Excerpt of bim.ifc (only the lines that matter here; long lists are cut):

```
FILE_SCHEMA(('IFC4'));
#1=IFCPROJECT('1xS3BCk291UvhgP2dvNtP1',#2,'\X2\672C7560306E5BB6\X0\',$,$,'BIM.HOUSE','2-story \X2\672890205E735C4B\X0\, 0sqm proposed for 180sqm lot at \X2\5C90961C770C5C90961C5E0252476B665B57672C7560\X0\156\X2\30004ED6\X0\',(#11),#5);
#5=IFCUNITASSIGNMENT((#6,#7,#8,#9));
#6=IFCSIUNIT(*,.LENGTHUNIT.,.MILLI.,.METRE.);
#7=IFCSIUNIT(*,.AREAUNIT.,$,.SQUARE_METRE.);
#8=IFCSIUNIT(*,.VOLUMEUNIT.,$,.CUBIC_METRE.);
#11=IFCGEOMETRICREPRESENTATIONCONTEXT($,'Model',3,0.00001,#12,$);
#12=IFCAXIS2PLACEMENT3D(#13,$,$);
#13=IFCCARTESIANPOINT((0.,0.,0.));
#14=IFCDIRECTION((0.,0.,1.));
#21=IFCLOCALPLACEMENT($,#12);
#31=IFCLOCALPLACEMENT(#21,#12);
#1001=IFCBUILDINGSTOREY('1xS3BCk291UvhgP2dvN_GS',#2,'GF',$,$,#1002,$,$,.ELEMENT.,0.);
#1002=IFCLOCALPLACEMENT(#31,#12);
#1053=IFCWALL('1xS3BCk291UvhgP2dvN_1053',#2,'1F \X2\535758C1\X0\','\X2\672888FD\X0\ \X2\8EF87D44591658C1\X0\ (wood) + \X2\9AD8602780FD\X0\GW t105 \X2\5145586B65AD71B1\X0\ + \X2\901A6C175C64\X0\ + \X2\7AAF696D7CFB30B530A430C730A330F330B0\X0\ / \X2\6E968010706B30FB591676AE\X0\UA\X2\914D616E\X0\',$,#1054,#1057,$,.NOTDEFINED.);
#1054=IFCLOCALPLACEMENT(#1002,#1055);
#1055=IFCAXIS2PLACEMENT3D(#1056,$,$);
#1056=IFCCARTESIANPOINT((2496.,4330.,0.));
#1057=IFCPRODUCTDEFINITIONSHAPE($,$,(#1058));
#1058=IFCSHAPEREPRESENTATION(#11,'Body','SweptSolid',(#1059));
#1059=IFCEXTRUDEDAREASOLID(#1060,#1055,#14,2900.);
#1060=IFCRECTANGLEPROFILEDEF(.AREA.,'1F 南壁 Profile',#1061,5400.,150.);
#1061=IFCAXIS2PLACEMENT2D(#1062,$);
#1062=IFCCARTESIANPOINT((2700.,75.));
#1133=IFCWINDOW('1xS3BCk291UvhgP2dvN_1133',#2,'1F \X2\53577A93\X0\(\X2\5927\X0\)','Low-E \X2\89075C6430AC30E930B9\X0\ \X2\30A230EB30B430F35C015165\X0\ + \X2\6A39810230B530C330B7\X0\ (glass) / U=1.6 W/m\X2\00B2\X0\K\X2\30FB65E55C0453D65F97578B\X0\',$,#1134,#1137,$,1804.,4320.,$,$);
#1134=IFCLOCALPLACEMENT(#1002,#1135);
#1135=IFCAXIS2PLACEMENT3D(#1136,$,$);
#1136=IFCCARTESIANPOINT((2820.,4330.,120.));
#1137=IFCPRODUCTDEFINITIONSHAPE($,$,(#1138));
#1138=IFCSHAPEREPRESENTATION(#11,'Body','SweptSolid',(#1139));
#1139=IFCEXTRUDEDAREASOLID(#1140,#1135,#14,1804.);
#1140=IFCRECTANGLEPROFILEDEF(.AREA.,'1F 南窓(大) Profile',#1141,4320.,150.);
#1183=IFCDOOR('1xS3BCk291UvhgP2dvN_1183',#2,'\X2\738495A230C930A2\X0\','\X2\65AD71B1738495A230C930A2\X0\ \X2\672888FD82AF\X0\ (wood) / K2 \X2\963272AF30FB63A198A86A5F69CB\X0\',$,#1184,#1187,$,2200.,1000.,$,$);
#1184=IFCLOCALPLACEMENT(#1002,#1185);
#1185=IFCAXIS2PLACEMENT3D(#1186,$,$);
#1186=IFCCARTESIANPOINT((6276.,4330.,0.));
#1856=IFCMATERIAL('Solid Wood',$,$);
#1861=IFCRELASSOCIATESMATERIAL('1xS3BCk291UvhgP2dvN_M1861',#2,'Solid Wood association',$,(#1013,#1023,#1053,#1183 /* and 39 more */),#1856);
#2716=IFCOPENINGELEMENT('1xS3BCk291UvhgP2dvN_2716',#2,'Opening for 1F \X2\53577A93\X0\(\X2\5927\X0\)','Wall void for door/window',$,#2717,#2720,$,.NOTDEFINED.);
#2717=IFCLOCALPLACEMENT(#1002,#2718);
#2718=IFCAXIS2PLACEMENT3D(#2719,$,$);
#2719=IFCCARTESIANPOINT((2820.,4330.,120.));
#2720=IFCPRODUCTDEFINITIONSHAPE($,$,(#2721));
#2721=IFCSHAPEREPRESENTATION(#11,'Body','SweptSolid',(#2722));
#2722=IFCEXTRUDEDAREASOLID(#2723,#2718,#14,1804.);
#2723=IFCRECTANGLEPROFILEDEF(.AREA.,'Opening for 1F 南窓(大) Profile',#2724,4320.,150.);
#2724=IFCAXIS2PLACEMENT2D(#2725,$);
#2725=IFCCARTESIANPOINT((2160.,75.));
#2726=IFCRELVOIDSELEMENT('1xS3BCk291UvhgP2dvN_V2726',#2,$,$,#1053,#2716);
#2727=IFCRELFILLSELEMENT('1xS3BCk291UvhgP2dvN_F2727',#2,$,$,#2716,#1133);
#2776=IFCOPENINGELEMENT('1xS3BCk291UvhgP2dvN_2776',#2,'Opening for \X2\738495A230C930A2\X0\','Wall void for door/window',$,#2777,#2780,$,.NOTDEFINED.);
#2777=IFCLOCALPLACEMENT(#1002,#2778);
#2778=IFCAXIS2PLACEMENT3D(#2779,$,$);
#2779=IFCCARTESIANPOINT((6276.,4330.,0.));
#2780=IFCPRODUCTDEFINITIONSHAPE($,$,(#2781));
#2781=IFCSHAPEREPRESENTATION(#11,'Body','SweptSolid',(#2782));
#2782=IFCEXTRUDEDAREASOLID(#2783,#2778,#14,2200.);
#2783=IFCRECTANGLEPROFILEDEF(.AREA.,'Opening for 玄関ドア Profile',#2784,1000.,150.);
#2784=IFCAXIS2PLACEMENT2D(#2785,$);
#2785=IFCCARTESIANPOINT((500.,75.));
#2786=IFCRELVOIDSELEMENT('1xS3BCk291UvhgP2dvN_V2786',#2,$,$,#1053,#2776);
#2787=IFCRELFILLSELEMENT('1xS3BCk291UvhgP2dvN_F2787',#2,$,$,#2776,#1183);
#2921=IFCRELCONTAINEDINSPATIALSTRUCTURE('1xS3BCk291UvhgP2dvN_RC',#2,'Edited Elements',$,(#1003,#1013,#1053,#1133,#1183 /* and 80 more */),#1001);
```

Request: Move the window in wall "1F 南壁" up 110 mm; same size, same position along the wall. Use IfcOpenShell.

```python
import numpy as np
import ifcopenshell
import ifcopenshell.api.geometry
import ifcopenshell.util.placement
import ifcopenshell.util.unit

model = ifcopenshell.open("bim.ifc")
unit_scale = ifcopenshell.util.unit.calculate_unit_scale(model)

window = model.by_guid("1xS3BCk291UvhgP2dvN_1133")
opening = window.FillsVoids[0].RelatingOpeningElement
dz = 0.11 / unit_scale

shift = np.array([0.0, 0.0, dz])
# The window is not placed relative to its opening, so move both.
for product in (opening, window):
    matrix = ifcopenshell.util.placement.get_local_placement(product.ObjectPlacement)
    matrix[:3, 3] += shift
    ifcopenshell.api.geometry.edit_object_placement(model, product=product, matrix=matrix, is_si=False)

print(f"moved by {dz * unit_scale:+.3f} m")

model.write("bim_v2.ifc")
```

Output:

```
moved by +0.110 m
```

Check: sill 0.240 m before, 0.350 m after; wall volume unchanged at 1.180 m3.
